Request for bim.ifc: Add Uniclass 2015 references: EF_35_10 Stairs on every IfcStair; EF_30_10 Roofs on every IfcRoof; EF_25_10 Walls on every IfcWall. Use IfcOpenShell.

First a look at what the model holds.

```python
import ifcopenshell

model = ifcopenshell.open("bim.ifc")
print(model.schema)
print("classifications:", [c.Name for c in model.by_type("IfcClassification")])
for ifc_class in ("IfcDoor", "IfcRoof", "IfcStair", "IfcWall", "IfcWindow"):
    print(ifc_class, len(model.by_type(ifc_class)))
```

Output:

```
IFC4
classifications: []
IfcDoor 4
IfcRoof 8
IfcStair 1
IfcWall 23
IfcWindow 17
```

```python
import ifcopenshell
import ifcopenshell.api.classification

model = ifcopenshell.open("bim.ifc")

system = ifcopenshell.api.classification.add_classification(model, classification="Uniclass 2015")

codes = {
    "IfcStair": ("EF_35_10", "Stairs"),
    "IfcRoof": ("EF_30_10", "Roofs"),
    "IfcWall": ("EF_25_10", "Walls"),
}
for ifc_class, (code, name) in codes.items():
    products = model.by_type(ifc_class)
    ifcopenshell.api.classification.add_reference(
        model, products=products, classification=system, identification=code, name=name
    )
    print(code, len(products))

model.write("bim_edited.ifc")
```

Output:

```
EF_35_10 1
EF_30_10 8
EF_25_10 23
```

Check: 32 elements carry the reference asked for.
